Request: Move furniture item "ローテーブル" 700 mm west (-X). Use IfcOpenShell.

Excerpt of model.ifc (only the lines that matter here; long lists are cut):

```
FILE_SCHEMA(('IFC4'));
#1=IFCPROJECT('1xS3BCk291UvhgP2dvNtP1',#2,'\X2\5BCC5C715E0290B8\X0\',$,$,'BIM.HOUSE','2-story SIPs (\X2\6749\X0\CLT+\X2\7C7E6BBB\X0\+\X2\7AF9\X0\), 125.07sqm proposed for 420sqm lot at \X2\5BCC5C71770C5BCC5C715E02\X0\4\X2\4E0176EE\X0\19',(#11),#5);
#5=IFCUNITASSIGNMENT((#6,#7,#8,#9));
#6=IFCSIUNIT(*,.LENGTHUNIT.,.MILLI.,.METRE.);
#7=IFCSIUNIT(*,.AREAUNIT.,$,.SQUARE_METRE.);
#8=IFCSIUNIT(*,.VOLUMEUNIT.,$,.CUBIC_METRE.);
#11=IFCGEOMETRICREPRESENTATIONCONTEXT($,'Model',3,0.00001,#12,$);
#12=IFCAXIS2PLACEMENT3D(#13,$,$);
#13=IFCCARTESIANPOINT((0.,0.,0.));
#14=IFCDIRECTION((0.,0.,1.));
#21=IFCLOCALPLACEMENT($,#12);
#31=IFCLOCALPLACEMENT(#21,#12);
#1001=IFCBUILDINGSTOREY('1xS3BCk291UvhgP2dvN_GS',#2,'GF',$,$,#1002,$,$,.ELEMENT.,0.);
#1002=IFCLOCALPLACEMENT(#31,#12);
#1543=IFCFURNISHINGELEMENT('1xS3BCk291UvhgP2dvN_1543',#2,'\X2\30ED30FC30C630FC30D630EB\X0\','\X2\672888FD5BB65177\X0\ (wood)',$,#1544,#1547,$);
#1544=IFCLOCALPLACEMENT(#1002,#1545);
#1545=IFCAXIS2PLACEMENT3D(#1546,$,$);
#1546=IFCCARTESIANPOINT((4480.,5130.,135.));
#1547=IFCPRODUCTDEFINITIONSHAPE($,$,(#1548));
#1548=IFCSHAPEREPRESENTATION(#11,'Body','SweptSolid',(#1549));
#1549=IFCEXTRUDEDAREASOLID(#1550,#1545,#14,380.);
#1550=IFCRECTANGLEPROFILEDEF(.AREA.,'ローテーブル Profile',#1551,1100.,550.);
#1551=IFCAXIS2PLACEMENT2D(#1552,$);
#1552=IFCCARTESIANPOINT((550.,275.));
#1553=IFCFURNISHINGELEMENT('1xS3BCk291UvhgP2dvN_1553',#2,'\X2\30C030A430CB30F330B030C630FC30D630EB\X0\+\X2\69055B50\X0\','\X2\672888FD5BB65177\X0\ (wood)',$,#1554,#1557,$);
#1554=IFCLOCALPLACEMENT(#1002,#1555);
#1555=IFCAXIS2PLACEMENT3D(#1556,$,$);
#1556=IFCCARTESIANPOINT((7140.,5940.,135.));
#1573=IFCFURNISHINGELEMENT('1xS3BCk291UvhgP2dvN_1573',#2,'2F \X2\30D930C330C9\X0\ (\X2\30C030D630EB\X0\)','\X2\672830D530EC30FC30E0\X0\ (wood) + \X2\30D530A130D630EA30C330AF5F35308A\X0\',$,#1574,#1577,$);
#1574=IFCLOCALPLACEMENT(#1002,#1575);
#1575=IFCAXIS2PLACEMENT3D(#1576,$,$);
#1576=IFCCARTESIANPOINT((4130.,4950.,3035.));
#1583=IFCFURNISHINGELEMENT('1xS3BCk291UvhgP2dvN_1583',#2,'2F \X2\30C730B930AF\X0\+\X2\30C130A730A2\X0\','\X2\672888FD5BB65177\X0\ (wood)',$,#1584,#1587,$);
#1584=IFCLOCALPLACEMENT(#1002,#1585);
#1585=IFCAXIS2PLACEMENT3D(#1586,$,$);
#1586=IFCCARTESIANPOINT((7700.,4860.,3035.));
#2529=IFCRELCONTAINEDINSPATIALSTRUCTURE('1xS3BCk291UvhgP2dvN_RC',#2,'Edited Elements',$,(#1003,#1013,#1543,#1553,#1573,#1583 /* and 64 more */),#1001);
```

```python
import ifcopenshell
import ifcopenshell.api.geometry
import ifcopenshell.util.placement
import ifcopenshell.util.unit

model = ifcopenshell.open("model.ifc")
unit_scale = ifcopenshell.util.unit.calculate_unit_scale(model)

item = model.by_guid("1xS3BCk291UvhgP2dvN_1543")
matrix = ifcopenshell.util.placement.get_local_placement(item.ObjectPlacement)
matrix[0, 3] -= 0.7 / unit_scale
ifcopenshell.api.geometry.edit_object_placement(model, product=item, matrix=matrix, is_si=False)

print(ifcopenshell.util.placement.get_local_placement(item.ObjectPlacement).round(3) + 0.0)

model.write("model_rev.ifc")
```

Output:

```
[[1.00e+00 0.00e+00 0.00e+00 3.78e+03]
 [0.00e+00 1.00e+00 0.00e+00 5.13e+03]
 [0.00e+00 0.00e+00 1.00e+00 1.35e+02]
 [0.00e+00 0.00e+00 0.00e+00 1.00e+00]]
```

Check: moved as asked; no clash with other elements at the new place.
